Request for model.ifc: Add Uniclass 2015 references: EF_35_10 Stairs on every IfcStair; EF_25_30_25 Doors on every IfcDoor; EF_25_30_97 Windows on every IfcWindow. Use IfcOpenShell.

First a look at what the model holds.

```python
import ifcopenshell

model = ifcopenshell.open("model.ifc")
print(model.schema)
print("classifications:", [c.Name for c in model.by_type("IfcClassification")])
for ifc_class in ("IfcDoor", "IfcRoof", "IfcStair", "IfcWall", "IfcWindow"):
    print(ifc_class, len(model.by_type(ifc_class)))
```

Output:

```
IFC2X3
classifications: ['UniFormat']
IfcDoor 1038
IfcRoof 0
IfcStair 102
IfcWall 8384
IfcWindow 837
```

```python
import ifcopenshell
import ifcopenshell.api.classification

model = ifcopenshell.open("model.ifc")

# IFC2X3 requires Source and Edition and has no link from the project to the system.
system = model.create_entity("IfcClassification", Source="NBS", Edition="2015", Name="Uniclass 2015")

codes = {
    "IfcStair": ("EF_35_10", "Stairs"),
    "IfcDoor": ("EF_25_30_25", "Doors"),
    "IfcWindow": ("EF_25_30_97", "Windows"),
}
for ifc_class, (code, name) in codes.items():
    products = model.by_type(ifc_class)
    ifcopenshell.api.classification.add_reference(
        model, products=products, classification=system, identification=code, name=name
    )
    print(code, len(products))

model.write("model-out.ifc")
```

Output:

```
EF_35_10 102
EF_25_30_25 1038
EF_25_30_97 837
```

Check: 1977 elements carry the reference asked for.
